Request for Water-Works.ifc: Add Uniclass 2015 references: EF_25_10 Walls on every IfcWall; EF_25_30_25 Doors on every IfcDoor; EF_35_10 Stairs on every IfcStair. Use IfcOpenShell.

First a look at what the model holds.

```python
import ifcopenshell

model = ifcopenshell.open("Water-Works.ifc")
print(model.schema)
print("classifications:", [c.Name for c in model.by_type("IfcClassification")])
for ifc_class in ("IfcDoor", "IfcRoof", "IfcStair", "IfcWall", "IfcWindow"):
    print(ifc_class, len(model.by_type(ifc_class)))
```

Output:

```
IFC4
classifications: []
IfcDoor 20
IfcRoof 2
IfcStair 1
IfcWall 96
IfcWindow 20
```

```python
import ifcopenshell
import ifcopenshell.api.classification

model = ifcopenshell.open("Water-Works.ifc")

system = ifcopenshell.api.classification.add_classification(model, classification="Uniclass 2015")

codes = {
    "IfcWall": ("EF_25_10", "Walls"),
    "IfcDoor": ("EF_25_30_25", "Doors"),
    "IfcStair": ("EF_35_10", "Stairs"),
}
for ifc_class, (code, name) in codes.items():
    products = model.by_type(ifc_class)
    ifcopenshell.api.classification.add_reference(
        model, products=products, classification=system, identification=code, name=name
    )
    print(code, len(products))

model.write("Water-Works-out.ifc")
```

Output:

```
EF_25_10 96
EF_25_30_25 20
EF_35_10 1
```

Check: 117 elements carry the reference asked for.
